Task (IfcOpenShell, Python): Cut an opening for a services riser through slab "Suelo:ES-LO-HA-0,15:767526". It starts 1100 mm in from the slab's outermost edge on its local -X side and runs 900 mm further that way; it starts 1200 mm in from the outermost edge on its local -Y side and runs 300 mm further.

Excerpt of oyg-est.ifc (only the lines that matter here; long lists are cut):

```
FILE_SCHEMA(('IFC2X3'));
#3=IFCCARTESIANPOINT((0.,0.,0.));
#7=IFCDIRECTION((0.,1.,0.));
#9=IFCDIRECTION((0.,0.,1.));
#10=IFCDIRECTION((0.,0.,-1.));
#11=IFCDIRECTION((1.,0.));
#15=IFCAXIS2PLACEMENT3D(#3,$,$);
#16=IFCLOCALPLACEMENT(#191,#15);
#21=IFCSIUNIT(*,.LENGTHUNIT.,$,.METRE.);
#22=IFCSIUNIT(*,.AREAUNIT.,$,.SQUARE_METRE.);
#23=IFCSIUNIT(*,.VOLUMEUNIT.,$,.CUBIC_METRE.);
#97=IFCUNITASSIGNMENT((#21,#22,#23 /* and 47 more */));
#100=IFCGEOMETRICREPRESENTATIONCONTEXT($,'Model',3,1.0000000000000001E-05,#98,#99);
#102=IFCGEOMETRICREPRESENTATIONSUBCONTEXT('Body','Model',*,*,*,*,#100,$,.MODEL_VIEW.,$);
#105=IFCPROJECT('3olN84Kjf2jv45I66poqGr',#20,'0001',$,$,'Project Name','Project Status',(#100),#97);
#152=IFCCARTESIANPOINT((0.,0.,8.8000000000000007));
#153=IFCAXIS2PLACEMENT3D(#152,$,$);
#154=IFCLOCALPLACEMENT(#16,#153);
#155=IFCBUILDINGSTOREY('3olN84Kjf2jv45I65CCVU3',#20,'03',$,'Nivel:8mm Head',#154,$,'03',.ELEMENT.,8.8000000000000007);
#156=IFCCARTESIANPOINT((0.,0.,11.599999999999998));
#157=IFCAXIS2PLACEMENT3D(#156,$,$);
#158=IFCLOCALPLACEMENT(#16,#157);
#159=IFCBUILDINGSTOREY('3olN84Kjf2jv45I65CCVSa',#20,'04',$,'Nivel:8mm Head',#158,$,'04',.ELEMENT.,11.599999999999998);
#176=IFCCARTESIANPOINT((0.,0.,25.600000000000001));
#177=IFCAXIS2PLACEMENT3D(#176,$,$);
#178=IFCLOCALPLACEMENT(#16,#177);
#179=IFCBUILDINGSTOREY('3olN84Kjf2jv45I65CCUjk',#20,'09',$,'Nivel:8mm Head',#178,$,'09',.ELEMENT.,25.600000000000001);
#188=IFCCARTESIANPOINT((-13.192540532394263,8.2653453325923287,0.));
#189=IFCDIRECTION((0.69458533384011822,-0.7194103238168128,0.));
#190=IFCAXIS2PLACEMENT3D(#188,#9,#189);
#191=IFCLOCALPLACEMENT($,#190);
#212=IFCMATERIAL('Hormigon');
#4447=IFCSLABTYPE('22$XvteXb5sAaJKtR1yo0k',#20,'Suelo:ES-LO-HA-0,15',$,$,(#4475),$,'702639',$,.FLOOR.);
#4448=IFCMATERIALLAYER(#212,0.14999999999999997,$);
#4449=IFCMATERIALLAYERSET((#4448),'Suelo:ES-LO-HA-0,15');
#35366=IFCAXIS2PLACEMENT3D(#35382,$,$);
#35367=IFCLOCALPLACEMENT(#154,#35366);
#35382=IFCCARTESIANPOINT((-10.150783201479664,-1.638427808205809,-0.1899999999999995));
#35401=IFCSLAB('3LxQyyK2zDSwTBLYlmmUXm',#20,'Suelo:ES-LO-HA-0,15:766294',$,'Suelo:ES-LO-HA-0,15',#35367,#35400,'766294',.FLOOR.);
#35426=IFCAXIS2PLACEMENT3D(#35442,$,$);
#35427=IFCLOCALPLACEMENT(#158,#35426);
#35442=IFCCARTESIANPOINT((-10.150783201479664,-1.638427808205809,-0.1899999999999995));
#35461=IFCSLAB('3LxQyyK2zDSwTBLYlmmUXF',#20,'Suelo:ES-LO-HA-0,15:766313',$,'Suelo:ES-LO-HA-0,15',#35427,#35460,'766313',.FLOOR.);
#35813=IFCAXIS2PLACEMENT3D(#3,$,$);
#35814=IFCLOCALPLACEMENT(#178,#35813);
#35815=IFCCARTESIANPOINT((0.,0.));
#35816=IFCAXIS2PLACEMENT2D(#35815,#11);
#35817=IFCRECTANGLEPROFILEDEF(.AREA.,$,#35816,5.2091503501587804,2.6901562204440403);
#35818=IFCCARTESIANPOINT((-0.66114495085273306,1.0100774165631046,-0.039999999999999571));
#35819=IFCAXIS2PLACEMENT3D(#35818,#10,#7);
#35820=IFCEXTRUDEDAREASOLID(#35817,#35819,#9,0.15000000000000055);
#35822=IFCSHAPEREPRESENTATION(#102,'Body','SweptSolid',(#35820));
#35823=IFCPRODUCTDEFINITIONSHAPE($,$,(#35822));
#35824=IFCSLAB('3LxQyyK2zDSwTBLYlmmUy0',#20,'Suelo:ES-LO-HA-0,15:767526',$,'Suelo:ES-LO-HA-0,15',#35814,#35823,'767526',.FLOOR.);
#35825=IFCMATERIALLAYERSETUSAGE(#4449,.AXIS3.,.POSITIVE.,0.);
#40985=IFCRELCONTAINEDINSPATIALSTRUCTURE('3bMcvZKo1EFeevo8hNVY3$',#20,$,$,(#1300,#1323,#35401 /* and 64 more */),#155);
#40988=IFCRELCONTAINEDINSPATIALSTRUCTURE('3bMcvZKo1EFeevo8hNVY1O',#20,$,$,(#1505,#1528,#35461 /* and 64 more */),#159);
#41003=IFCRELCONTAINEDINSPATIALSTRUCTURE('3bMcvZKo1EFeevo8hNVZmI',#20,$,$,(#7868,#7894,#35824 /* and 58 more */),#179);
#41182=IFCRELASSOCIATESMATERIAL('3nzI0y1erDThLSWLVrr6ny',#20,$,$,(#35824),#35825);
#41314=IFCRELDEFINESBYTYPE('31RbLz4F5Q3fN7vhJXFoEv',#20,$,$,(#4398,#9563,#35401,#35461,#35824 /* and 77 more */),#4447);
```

```python
import numpy as np
import ifcopenshell
import ifcopenshell.api.feature
import ifcopenshell.api.geometry
import ifcopenshell.api.root
import ifcopenshell.geom
import ifcopenshell.util.placement
import ifcopenshell.util.representation
import ifcopenshell.util.shape
import ifcopenshell.util.unit

model = ifcopenshell.open("oyg-est.ifc")
unit_scale = ifcopenshell.util.unit.calculate_unit_scale(model)
settings = ifcopenshell.geom.settings()


def volume(element):
    """Net volume in cubic metres, openings subtracted."""
    shape = ifcopenshell.geom.create_shape(settings, element)
    return ifcopenshell.util.shape.get_volume(shape.geometry)


slab = model.by_guid("3LxQyyK2zDSwTBLYlmmUy0")
before = volume(slab)

# Extent in the slab's own axes, in metres. The edges named are its -X and -Y sides.
slab_shape = ifcopenshell.geom.create_shape(settings, slab)
vertices = ifcopenshell.util.shape.get_vertices(slab_shape.geometry)
x_min, y_min, bottom = vertices.min(axis=0)
top = vertices[:, 2].max()

opening = ifcopenshell.api.root.create_entity(model, ifc_class="IfcOpeningElement", name="Services riser opening")
context = ifcopenshell.util.representation.get_context(model, "Model", "Body", "MODEL_VIEW")
width, depth = 0.9, 0.3
outline = [(0.0, 0.0), (width, 0.0), (width, depth), (0.0, depth), (0.0, 0.0)]
# Overshoot both faces by 50 mm so the cut is clean.
shape = ifcopenshell.api.geometry.add_slab_representation(
    model, context=context, depth=top - bottom + 0.1, polyline=outline
)
ifcopenshell.api.geometry.assign_representation(model, product=opening, representation=shape)

matrix = ifcopenshell.util.placement.get_local_placement(slab.ObjectPlacement)
matrix[:, 3] = matrix @ np.append(np.array([x_min + 1.1, y_min + 1.2, bottom - 0.05]) / unit_scale, 1.0)
ifcopenshell.api.geometry.edit_object_placement(model, product=opening, matrix=matrix, is_si=False)
ifcopenshell.api.feature.add_feature(model, feature=opening, element=slab)

after = volume(slab)

print(f"slab volume {before:.3f} -> {after:.3f} m3")

model.write("oyg-est_edited.ifc")
```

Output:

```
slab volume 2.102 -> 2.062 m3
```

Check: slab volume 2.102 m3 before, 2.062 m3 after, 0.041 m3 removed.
